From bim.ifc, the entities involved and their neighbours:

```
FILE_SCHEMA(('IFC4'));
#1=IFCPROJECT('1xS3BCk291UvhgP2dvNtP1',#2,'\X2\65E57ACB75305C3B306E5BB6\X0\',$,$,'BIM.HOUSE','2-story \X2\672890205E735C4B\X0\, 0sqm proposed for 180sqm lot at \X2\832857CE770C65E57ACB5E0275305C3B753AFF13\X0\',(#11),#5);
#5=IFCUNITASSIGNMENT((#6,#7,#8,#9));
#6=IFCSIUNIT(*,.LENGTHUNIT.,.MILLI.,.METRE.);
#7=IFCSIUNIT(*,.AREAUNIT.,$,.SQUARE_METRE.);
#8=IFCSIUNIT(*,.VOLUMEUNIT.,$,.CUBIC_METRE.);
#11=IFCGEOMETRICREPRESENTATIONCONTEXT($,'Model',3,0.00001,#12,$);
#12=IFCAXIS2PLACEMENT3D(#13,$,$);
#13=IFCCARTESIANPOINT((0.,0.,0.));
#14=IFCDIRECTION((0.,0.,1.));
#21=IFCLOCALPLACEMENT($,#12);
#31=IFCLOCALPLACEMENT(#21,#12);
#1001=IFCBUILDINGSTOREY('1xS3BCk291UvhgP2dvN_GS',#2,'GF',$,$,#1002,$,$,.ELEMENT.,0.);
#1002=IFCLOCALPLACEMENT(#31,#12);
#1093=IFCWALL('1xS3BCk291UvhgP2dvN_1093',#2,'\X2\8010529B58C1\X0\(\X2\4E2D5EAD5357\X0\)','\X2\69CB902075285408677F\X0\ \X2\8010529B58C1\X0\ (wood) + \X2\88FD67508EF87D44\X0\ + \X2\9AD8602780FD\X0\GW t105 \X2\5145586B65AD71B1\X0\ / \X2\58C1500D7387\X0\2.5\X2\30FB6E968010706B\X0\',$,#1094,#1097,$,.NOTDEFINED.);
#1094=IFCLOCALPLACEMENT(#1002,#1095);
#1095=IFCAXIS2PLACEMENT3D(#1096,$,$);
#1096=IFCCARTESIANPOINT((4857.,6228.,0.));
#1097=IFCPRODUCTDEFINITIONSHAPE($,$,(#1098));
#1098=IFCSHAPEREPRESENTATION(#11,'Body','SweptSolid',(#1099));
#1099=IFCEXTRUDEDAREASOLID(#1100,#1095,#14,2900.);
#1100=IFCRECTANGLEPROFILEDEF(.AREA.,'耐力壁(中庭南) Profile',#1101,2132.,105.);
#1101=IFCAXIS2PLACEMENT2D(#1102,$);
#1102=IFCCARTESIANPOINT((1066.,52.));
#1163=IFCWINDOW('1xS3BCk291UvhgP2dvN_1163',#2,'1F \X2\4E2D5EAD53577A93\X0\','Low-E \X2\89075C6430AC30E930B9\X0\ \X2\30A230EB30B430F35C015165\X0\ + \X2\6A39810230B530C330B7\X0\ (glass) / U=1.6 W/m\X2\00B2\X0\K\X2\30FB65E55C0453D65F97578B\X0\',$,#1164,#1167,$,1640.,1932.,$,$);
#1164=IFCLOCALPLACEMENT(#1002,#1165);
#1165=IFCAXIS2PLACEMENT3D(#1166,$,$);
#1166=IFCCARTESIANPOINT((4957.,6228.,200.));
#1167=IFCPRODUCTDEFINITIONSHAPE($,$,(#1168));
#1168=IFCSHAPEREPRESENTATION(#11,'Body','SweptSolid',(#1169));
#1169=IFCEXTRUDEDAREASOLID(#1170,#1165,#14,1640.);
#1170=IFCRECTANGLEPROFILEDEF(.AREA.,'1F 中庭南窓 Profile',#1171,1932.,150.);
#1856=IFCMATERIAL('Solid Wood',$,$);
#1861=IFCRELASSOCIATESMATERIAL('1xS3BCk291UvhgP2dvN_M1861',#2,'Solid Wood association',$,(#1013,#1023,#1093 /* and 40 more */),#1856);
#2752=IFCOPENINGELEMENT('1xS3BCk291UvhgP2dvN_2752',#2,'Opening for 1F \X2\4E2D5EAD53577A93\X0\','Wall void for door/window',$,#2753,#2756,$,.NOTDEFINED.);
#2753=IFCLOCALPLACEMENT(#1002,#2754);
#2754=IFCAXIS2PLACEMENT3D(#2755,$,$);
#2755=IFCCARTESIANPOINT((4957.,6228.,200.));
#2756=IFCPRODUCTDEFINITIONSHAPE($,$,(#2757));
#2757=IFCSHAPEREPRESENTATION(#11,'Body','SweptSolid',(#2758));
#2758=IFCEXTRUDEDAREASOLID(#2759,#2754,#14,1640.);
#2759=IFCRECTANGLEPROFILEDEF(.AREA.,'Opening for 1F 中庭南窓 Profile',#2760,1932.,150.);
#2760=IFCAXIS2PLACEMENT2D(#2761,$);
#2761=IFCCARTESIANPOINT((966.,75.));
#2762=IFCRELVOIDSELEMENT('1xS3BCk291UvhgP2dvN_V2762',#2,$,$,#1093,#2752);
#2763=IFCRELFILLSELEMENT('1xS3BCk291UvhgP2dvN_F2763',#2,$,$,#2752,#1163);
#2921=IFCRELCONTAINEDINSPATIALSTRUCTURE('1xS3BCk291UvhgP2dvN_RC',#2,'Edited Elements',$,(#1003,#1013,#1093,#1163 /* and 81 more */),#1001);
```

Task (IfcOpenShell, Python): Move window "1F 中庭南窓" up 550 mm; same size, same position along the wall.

```python
import numpy as np
import ifcopenshell
import ifcopenshell.api.geometry
import ifcopenshell.util.placement
import ifcopenshell.util.unit

model = ifcopenshell.open("bim.ifc")
unit_scale = ifcopenshell.util.unit.calculate_unit_scale(model)

window = model.by_guid("1xS3BCk291UvhgP2dvN_1163")
opening = window.FillsVoids[0].RelatingOpeningElement
dz = 0.55 / unit_scale

shift = np.array([0.0, 0.0, dz])
# The window is not placed relative to its opening, so move both.
for product in (opening, window):
    matrix = ifcopenshell.util.placement.get_local_placement(product.ObjectPlacement)
    matrix[:3, 3] += shift
    ifcopenshell.api.geometry.edit_object_placement(model, product=product, matrix=matrix, is_si=False)

print(f"moved by {dz * unit_scale:+.3f} m")

model.write("bim_v2.ifc")
```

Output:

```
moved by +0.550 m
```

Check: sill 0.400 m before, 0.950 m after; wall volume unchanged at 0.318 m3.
